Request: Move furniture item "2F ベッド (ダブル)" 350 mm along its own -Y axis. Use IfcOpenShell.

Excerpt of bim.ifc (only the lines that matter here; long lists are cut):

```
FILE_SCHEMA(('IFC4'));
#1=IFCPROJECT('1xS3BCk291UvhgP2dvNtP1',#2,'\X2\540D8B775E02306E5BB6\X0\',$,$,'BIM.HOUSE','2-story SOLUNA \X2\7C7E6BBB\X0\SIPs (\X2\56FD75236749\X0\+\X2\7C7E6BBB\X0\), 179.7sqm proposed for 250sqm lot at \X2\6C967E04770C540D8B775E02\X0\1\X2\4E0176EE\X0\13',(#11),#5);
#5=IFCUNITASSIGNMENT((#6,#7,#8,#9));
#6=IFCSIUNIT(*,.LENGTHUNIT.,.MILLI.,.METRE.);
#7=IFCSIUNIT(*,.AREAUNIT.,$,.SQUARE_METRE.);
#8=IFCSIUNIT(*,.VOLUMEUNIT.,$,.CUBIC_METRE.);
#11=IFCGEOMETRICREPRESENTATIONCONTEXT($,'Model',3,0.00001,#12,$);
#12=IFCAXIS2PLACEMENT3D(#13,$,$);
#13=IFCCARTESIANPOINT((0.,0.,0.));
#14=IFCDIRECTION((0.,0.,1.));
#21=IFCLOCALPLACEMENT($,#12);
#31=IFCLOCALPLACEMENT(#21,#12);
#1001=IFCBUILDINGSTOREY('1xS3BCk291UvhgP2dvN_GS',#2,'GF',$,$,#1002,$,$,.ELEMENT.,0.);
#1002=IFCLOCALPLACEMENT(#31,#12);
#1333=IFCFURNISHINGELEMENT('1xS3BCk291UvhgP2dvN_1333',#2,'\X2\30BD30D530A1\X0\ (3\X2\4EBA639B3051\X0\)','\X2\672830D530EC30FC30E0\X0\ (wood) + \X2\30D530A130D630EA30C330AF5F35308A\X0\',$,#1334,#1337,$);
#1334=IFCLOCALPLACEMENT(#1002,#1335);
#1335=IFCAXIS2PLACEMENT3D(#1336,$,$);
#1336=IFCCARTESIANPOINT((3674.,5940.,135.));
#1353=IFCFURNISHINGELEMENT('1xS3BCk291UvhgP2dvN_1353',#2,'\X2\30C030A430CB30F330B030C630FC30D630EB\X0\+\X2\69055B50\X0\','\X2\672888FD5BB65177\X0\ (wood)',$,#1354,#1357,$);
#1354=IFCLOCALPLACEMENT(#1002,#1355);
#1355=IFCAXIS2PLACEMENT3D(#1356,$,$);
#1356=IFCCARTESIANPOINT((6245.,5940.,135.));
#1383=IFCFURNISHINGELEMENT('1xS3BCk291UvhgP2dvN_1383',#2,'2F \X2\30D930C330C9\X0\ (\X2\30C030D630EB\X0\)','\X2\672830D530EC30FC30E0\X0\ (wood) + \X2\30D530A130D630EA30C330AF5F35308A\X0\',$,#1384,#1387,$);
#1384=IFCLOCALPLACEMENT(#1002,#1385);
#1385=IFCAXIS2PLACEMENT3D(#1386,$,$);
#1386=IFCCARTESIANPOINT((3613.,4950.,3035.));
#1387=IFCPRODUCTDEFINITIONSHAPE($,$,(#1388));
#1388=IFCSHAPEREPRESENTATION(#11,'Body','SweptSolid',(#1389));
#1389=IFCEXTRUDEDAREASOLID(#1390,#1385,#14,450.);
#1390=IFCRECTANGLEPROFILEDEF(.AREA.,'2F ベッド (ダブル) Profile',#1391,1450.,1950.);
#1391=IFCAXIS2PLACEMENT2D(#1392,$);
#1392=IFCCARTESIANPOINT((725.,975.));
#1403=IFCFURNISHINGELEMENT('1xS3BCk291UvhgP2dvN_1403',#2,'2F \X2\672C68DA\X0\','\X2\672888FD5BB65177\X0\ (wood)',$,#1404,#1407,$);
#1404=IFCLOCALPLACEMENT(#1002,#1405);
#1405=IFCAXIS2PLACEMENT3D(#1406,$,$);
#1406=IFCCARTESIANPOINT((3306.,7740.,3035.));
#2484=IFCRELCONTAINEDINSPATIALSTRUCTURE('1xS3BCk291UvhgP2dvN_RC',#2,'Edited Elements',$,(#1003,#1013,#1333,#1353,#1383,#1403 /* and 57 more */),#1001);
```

```python
import ifcopenshell
import ifcopenshell.api.geometry
import ifcopenshell.util.placement
import ifcopenshell.util.unit

model = ifcopenshell.open("bim.ifc")
unit_scale = ifcopenshell.util.unit.calculate_unit_scale(model)

item = model.by_guid("1xS3BCk291UvhgP2dvN_1383")
matrix = ifcopenshell.util.placement.get_local_placement(item.ObjectPlacement)
matrix[:3, 3] -= matrix[:3, 1] * 0.35 / unit_scale
ifcopenshell.api.geometry.edit_object_placement(model, product=item, matrix=matrix, is_si=False)

print(ifcopenshell.util.placement.get_local_placement(item.ObjectPlacement).round(3) + 0.0)

model.write("bim_edited.ifc")
```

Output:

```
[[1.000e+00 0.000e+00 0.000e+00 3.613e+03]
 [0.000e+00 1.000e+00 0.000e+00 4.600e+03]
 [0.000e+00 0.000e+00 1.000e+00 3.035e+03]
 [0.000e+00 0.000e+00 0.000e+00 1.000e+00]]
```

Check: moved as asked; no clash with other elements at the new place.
